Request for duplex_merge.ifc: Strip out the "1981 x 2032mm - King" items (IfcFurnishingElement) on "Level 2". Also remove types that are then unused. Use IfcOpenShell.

First a look at what the model holds.

```python
import ifcopenshell
import ifcopenshell.util.element

model = ifcopenshell.open("duplex_merge.ifc")
print(model.schema)
storey = next(s for s in model.by_type("IfcBuildingStorey") if s.Name == "Level 2")
furniture = [e for e in ifcopenshell.util.element.get_decomposition(storey) if e.is_a("IfcFurnishingElement")]
seen = {}
for e in furniture:
    element_type = ifcopenshell.util.element.get_type(e)
    name = element_type.Name if element_type not in (None, e) else None
    seen[name] = seen.get(name, 0) + 1
for name, count in sorted(seen.items(), key=str):
    print(count, "x", name)
```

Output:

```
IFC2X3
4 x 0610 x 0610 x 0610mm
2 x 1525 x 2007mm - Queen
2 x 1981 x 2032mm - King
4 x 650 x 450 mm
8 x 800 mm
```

```python
import ifcopenshell
import ifcopenshell.api.root
import ifcopenshell.util.element

model = ifcopenshell.open("duplex_merge.ifc")

storey = next(s for s in model.by_type("IfcBuildingStorey") if s.Name == "Level 2")
furniture = [e for e in ifcopenshell.util.element.get_decomposition(storey) if e.is_a("IfcFurnishingElement")]
targets = [e for e in furniture if (t := ifcopenshell.util.element.get_type(e)) not in (None, e) and t.Name == "1981 x 2032mm - King"]
types = {ifcopenshell.util.element.get_type(e) for e in targets} - {None, *targets}

for e in targets:
    ifcopenshell.api.root.remove_product(model, product=e)
print(len(targets), "removed")

unused = [t for t in types if not ifcopenshell.util.element.get_types(t)]
for t in unused:
    ifcopenshell.api.root.remove_product(model, product=t)
print(len(unused), "unused types removed")

model.write("duplex_merge_rev.ifc")
```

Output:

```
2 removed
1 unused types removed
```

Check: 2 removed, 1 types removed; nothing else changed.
